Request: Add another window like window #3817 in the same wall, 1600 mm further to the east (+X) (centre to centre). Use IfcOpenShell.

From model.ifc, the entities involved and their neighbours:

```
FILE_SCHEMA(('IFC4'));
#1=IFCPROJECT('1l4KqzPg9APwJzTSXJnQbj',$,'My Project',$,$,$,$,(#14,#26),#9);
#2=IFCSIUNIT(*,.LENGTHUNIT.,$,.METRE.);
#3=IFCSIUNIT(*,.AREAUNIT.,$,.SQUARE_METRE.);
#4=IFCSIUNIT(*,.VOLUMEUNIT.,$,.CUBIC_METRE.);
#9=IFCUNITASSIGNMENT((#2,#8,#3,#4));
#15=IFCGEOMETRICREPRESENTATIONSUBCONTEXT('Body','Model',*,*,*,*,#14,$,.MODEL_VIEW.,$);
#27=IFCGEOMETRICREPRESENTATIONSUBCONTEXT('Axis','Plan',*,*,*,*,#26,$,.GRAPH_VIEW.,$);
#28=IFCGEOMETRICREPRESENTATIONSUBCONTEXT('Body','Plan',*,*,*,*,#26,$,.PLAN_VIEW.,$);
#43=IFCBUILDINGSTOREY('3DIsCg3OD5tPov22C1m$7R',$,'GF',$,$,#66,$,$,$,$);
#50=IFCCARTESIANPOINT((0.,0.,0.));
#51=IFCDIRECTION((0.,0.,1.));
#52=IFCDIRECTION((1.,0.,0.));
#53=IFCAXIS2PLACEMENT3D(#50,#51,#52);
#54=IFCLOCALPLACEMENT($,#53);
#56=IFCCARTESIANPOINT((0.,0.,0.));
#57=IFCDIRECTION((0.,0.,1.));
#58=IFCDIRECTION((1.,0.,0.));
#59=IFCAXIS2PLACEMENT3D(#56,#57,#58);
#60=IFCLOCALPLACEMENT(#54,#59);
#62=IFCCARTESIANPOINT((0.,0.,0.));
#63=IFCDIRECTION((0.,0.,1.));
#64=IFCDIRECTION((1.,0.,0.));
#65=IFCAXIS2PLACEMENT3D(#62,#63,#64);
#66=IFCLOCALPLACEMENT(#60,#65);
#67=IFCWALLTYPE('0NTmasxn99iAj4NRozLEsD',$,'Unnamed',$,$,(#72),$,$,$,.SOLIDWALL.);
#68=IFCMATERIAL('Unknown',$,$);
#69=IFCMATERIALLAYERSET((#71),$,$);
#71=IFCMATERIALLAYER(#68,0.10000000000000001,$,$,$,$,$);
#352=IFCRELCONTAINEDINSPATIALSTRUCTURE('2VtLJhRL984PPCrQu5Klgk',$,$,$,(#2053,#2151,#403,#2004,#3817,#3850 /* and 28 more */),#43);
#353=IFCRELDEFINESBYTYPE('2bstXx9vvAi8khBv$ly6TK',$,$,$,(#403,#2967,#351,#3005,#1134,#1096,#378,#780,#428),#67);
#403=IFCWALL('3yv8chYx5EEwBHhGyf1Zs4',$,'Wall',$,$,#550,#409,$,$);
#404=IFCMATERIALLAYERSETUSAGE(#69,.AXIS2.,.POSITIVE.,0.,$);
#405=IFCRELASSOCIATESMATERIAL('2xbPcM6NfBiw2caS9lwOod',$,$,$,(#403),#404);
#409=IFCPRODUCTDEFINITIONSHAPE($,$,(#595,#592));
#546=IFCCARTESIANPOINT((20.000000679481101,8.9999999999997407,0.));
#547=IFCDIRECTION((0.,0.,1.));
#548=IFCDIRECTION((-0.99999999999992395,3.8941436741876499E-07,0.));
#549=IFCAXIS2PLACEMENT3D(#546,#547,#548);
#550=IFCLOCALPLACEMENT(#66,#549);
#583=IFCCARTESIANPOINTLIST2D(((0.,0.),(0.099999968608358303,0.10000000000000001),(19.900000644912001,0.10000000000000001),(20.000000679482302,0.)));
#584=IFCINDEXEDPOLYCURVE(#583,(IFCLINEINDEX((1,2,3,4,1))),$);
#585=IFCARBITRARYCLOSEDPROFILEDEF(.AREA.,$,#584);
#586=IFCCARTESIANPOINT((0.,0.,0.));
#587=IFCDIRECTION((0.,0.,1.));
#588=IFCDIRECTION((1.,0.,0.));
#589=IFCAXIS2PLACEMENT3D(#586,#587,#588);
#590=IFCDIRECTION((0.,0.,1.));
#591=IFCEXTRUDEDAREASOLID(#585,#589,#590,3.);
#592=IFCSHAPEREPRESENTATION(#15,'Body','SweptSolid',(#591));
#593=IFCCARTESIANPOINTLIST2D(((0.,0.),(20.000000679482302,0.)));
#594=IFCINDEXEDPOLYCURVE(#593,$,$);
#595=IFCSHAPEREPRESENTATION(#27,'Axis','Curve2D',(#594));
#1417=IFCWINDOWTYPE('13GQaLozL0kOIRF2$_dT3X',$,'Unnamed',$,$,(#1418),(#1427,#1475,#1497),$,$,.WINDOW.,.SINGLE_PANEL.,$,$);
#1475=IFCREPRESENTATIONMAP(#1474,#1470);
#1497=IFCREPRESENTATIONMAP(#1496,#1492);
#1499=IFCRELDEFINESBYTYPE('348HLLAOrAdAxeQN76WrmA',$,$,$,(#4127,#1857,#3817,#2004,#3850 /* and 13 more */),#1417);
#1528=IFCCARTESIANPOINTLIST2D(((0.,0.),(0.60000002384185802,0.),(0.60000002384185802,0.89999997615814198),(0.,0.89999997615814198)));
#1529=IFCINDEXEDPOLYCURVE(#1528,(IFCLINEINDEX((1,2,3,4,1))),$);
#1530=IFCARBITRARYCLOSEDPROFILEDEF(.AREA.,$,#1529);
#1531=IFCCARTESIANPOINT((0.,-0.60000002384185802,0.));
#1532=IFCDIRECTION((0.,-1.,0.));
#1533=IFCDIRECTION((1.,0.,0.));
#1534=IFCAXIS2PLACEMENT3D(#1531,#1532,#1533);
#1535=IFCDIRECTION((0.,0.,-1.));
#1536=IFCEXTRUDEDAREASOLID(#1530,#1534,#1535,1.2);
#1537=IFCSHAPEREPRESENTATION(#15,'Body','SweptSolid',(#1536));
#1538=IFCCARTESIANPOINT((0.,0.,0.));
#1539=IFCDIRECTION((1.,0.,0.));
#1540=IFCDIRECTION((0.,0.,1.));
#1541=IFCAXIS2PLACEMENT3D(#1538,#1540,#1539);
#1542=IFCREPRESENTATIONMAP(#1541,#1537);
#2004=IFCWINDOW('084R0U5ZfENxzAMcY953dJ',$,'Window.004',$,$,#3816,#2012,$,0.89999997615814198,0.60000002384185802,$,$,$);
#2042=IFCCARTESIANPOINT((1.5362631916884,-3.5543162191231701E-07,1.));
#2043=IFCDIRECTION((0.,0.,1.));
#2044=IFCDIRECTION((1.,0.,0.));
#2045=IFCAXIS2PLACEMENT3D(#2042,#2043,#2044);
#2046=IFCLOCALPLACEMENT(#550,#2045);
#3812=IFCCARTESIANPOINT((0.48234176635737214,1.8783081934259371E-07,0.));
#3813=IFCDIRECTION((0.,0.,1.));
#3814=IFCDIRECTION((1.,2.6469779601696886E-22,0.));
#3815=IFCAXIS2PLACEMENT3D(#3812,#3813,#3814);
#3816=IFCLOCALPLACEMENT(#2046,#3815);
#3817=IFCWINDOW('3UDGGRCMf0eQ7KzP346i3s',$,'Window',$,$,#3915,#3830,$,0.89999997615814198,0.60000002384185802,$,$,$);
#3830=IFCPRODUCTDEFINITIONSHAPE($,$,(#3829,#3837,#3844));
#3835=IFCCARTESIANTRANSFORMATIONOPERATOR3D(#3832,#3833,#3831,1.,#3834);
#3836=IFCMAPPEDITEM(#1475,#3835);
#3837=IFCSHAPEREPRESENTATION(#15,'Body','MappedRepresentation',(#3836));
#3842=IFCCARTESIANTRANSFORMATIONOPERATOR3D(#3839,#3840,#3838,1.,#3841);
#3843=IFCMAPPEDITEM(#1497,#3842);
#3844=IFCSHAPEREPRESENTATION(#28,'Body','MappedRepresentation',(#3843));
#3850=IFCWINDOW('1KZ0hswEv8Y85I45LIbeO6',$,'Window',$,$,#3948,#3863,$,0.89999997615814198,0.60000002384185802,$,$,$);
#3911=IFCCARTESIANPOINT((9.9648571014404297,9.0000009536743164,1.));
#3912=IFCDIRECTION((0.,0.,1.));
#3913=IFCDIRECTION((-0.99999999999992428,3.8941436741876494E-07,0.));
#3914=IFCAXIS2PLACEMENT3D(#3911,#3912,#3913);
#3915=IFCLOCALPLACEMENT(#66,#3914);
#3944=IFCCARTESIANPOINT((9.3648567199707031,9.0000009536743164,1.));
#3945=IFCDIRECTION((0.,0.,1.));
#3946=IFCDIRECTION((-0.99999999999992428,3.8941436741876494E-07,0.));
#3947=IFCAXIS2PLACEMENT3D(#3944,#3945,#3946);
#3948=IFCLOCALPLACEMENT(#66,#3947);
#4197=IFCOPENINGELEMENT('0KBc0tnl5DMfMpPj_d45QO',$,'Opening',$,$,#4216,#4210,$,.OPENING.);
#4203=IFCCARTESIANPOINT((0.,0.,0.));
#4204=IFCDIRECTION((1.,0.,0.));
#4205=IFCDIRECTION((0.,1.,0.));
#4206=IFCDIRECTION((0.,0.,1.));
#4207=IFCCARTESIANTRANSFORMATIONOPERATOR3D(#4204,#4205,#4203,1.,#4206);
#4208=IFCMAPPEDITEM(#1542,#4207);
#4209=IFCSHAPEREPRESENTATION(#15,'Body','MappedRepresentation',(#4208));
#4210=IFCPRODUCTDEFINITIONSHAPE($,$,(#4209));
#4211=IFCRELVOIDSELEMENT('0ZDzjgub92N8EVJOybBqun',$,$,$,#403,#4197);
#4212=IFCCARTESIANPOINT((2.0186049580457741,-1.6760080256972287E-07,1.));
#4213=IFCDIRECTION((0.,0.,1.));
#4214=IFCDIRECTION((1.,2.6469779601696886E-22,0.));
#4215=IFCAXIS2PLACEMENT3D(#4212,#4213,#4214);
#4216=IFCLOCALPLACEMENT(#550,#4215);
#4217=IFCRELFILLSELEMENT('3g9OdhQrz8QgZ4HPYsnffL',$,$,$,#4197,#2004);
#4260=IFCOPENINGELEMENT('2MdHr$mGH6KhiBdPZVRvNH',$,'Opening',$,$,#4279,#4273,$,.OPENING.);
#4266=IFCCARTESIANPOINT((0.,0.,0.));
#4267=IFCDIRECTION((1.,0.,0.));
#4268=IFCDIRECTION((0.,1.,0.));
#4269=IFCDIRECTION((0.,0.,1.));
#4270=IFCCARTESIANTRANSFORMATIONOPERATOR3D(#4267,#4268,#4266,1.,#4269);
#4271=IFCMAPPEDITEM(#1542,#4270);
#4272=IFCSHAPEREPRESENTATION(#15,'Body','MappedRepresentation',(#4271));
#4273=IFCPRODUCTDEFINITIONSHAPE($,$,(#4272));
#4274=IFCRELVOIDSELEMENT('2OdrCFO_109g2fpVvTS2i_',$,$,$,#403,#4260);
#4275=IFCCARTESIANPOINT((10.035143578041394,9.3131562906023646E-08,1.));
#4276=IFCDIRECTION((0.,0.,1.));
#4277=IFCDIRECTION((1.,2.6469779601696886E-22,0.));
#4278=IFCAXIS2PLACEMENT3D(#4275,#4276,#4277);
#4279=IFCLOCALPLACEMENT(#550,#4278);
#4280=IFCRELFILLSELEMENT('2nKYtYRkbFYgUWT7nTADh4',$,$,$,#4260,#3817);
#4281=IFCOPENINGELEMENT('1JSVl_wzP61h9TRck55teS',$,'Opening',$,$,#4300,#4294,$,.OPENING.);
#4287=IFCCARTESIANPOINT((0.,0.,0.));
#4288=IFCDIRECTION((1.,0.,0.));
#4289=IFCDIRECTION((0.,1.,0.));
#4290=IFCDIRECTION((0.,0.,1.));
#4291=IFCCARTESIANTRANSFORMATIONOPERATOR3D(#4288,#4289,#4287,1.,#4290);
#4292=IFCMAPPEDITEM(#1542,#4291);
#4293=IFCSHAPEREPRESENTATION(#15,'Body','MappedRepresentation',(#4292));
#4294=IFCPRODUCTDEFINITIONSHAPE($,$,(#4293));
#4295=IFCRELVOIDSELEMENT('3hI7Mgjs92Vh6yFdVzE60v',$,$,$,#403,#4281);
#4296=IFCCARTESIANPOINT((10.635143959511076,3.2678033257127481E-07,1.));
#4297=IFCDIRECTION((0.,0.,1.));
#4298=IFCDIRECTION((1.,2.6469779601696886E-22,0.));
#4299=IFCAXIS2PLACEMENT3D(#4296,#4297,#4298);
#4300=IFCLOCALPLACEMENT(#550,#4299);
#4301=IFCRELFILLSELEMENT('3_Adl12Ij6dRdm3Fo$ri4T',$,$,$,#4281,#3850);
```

```python
import ifcopenshell
import ifcopenshell.api.feature
import ifcopenshell.api.geometry
import ifcopenshell.api.root
import ifcopenshell.geom
import ifcopenshell.util.element
import ifcopenshell.util.placement
import ifcopenshell.util.shape

model = ifcopenshell.open("model.ifc")
settings = ifcopenshell.geom.settings()


def volume(element):
    """Net volume in cubic metres, openings subtracted."""
    shape = ifcopenshell.geom.create_shape(settings, element)
    return ifcopenshell.util.shape.get_volume(shape.geometry)


window = model.by_guid("3UDGGRCMf0eQ7KzP346i3s")
opening = window.FillsVoids[0].RelatingOpeningElement
wall = opening.VoidsElements[0].RelatingBuildingElement
before = volume(wall)
shift = ifcopenshell.util.placement.get_local_placement(wall.ObjectPlacement)[:3, 0] * -1.6

# copy_class copies the void relationship, type, container and properties, but no geometry.
new_opening = ifcopenshell.api.root.copy_class(model, product=opening)
new_opening.Representation = ifcopenshell.util.element.copy_deep(
    model, opening.Representation, exclude=["IfcGeometricRepresentationContext", "IfcRepresentationMap"]
)
new_window = ifcopenshell.api.root.copy_class(model, product=window)
new_window.Representation = ifcopenshell.util.element.copy_deep(
    model, window.Representation, exclude=["IfcGeometricRepresentationContext", "IfcRepresentationMap"]
)
ifcopenshell.api.feature.add_filling(model, opening=new_opening, element=new_window)

for old, new in ((opening, new_opening), (window, new_window)):
    matrix = ifcopenshell.util.placement.get_local_placement(old.ObjectPlacement)
    matrix[:3, 3] += shift
    ifcopenshell.api.geometry.edit_object_placement(model, product=new, matrix=matrix, is_si=False)

after = volume(wall)

print(f"wall volume {before:.3f} -> {after:.3f} m3")

model.write("model_rev.ifc")
```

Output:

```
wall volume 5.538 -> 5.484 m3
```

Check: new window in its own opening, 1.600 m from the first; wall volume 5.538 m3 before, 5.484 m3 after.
